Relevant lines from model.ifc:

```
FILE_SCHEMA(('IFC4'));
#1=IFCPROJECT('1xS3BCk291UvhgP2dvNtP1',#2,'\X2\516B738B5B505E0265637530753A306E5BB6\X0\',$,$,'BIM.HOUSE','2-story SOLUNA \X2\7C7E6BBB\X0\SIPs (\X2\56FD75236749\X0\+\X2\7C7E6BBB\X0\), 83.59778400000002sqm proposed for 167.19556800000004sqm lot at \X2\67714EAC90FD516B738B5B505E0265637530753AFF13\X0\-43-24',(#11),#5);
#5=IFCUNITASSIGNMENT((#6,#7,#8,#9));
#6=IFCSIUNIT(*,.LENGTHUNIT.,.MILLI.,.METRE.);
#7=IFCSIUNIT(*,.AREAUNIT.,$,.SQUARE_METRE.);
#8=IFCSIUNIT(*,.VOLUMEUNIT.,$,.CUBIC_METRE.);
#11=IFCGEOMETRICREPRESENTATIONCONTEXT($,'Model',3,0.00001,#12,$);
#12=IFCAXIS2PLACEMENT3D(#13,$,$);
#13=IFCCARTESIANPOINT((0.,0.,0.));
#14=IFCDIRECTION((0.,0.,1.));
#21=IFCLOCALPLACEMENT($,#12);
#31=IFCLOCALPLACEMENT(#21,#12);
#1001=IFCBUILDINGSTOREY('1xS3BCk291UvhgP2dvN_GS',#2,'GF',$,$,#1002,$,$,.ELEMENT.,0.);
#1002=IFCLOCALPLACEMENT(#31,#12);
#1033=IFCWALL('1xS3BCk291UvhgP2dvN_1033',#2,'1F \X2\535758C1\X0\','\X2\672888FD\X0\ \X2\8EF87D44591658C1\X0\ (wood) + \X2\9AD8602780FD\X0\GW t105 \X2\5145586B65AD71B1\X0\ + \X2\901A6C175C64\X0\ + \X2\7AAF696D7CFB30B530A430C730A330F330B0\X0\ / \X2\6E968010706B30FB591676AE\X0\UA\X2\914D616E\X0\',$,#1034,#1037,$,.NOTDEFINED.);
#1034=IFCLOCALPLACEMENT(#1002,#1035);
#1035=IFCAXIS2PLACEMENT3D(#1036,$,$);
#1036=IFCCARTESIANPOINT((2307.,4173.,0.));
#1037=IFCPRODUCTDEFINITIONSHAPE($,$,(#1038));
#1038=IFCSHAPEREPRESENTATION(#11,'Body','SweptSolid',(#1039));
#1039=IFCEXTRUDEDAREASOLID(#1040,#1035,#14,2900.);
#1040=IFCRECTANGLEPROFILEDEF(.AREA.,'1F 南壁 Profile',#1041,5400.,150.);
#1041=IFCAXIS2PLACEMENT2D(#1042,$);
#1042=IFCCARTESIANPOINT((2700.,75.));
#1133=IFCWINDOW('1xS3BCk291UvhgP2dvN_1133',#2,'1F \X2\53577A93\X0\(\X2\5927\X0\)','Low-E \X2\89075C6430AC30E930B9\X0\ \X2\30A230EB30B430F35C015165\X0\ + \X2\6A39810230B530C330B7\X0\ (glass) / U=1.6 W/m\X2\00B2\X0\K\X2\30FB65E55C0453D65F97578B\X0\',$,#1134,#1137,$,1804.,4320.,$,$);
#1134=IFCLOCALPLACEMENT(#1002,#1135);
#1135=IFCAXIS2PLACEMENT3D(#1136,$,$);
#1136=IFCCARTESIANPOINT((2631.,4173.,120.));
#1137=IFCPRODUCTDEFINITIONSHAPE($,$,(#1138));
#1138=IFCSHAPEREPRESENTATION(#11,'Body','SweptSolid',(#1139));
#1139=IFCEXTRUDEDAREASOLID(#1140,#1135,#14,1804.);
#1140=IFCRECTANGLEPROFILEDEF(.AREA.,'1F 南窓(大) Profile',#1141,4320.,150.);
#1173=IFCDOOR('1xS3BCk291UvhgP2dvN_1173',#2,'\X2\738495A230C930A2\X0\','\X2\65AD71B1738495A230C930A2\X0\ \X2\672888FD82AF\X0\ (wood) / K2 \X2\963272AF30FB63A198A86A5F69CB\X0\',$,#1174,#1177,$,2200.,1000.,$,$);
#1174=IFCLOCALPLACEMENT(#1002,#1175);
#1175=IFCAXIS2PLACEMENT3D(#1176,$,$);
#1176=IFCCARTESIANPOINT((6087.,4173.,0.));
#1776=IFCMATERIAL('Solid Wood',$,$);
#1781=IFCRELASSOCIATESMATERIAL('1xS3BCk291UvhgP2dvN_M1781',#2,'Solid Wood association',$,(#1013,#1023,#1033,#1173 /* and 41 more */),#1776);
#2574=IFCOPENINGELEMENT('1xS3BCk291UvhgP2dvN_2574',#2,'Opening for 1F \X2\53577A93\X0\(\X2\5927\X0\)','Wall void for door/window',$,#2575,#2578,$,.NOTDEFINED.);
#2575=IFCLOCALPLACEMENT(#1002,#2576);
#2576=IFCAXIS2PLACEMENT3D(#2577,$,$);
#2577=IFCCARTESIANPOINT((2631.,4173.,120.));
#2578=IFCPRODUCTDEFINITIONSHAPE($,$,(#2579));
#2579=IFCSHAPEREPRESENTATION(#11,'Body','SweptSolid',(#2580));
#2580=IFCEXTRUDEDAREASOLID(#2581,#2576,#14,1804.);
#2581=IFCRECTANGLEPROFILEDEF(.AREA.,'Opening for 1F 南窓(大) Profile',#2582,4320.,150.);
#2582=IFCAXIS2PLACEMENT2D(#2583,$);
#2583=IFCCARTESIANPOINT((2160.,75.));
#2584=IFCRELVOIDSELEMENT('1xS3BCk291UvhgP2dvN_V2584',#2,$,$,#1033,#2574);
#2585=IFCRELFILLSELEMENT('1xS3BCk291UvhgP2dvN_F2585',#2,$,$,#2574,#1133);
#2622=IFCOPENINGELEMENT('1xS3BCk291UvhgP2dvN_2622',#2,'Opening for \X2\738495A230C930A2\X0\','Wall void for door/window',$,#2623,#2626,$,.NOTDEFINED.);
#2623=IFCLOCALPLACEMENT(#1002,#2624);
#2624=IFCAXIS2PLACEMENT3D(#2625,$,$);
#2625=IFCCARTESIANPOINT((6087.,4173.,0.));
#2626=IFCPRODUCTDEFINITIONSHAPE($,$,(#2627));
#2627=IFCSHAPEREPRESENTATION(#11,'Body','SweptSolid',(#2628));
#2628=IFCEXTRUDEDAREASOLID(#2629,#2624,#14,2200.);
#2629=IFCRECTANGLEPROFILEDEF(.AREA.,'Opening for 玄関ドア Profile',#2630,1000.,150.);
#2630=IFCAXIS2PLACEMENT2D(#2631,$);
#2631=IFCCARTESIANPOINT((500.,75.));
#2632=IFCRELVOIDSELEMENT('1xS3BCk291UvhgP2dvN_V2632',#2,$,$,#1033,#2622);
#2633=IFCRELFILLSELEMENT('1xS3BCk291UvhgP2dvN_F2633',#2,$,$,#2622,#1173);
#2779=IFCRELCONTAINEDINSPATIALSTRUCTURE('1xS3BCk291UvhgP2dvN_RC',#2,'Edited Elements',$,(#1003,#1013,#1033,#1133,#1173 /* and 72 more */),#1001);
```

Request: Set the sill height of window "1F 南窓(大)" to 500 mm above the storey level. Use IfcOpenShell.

```python
import numpy as np
import ifcopenshell
import ifcopenshell.api.geometry
import ifcopenshell.geom
import ifcopenshell.util.element
import ifcopenshell.util.placement
import ifcopenshell.util.shape
import ifcopenshell.util.unit

model = ifcopenshell.open("model.ifc")
unit_scale = ifcopenshell.util.unit.calculate_unit_scale(model)

window = model.by_guid("1xS3BCk291UvhgP2dvN_1133")
opening = window.FillsVoids[0].RelatingOpeningElement
storey = ifcopenshell.util.element.get_container(window, ifc_class="IfcBuildingStorey")
level = ifcopenshell.util.placement.get_local_placement(storey.ObjectPlacement)[2, 3]

# The opening's origin need not be at the sill, so measure its lowest point.
shape = ifcopenshell.geom.create_shape(ifcopenshell.geom.settings(), opening)
bottom = ifcopenshell.util.shape.get_shape_bottom_elevation(shape, shape.geometry) / unit_scale
dz = level + 500.0 - bottom

shift = np.array([0.0, 0.0, dz])
# The window is not placed relative to its opening, so move both.
for product in (opening, window):
    matrix = ifcopenshell.util.placement.get_local_placement(product.ObjectPlacement)
    matrix[:3, 3] += shift
    ifcopenshell.api.geometry.edit_object_placement(model, product=product, matrix=matrix, is_si=False)

print(f"moved by {dz * unit_scale:+.3f} m")

model.write("model-out.ifc")
```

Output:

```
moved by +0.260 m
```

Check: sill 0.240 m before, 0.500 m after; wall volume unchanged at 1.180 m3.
